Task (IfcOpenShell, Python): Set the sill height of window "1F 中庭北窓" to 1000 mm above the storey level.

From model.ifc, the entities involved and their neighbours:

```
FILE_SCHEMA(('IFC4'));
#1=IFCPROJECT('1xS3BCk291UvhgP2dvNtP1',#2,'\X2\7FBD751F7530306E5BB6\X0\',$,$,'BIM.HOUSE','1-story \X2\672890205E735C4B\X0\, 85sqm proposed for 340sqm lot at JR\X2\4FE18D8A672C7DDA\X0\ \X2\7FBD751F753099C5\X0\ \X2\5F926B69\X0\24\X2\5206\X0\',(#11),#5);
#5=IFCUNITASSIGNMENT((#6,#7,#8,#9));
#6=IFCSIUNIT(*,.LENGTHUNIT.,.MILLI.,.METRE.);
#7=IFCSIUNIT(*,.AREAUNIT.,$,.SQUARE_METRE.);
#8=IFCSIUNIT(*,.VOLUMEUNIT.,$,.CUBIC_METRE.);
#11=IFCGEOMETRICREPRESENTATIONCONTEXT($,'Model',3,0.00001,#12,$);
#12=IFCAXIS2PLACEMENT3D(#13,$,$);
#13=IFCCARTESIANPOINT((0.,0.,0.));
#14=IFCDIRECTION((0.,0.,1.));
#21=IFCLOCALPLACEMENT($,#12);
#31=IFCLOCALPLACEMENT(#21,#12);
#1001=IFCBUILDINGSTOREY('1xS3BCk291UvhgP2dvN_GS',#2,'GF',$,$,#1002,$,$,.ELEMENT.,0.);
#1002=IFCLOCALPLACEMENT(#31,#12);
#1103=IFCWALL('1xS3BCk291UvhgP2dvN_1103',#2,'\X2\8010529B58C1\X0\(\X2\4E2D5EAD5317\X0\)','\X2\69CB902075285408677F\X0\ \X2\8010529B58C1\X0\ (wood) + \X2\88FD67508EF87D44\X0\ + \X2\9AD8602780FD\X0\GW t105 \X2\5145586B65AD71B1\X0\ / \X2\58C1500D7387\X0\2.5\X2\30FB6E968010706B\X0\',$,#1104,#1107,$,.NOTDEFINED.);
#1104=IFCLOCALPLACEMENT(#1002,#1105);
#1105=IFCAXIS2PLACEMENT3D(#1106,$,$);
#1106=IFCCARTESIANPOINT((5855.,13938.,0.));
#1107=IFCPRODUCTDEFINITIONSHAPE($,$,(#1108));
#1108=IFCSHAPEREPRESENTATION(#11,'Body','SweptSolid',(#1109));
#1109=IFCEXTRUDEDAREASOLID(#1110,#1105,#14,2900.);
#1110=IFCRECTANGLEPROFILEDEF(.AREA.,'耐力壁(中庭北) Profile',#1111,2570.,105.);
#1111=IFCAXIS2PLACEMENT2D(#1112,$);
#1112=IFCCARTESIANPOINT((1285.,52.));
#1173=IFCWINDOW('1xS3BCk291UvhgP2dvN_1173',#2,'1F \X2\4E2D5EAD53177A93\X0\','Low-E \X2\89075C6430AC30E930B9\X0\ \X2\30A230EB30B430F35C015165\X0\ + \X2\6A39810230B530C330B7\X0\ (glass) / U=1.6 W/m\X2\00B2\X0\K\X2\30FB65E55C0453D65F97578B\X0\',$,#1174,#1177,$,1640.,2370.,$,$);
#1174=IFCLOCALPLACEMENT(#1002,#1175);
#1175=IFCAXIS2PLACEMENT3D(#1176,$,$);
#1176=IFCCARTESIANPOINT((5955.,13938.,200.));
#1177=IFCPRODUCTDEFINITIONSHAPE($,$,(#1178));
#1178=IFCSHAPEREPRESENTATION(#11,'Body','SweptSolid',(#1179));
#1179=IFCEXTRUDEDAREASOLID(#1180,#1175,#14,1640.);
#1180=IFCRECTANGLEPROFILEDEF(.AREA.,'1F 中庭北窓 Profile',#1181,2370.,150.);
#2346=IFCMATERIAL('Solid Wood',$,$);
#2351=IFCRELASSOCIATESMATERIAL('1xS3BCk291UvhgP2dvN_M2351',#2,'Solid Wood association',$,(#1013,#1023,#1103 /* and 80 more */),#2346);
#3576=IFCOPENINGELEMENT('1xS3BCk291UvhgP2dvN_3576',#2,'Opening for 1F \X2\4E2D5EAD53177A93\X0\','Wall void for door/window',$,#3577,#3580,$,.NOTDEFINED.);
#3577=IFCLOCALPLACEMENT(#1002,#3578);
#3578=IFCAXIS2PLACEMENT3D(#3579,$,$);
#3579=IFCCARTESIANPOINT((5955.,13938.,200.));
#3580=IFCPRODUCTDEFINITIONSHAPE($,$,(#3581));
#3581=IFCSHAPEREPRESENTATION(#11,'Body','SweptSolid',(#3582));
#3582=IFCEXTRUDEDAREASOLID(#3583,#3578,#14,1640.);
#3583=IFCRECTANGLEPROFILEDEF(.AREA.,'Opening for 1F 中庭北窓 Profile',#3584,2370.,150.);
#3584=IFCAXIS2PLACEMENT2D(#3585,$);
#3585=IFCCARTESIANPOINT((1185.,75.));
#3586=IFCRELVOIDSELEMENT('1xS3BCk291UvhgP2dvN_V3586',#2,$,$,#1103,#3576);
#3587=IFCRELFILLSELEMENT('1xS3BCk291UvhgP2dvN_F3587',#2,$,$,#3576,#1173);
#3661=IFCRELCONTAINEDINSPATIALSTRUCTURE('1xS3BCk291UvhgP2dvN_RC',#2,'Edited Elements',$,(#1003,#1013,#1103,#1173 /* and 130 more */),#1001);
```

```python
import numpy as np
import ifcopenshell
import ifcopenshell.api.geometry
import ifcopenshell.geom
import ifcopenshell.util.element
import ifcopenshell.util.placement
import ifcopenshell.util.shape
import ifcopenshell.util.unit

model = ifcopenshell.open("model.ifc")
unit_scale = ifcopenshell.util.unit.calculate_unit_scale(model)

window = model.by_guid("1xS3BCk291UvhgP2dvN_1173")
opening = window.FillsVoids[0].RelatingOpeningElement
storey = ifcopenshell.util.element.get_container(window, ifc_class="IfcBuildingStorey")
level = ifcopenshell.util.placement.get_local_placement(storey.ObjectPlacement)[2, 3]

# The opening's origin need not be at the sill, so measure its lowest point.
shape = ifcopenshell.geom.create_shape(ifcopenshell.geom.settings(), opening)
bottom = ifcopenshell.util.shape.get_shape_bottom_elevation(shape, shape.geometry) / unit_scale
dz = level + 1 / unit_scale - bottom

shift = np.array([0.0, 0.0, dz])
# The window is not placed relative to its opening, so move both.
for product in (opening, window):
    matrix = ifcopenshell.util.placement.get_local_placement(product.ObjectPlacement)
    matrix[:3, 3] += shift
    ifcopenshell.api.geometry.edit_object_placement(model, product=product, matrix=matrix, is_si=False)

print(f"moved by {dz * unit_scale:+.3f} m")

model.write("model_v2.ifc")
```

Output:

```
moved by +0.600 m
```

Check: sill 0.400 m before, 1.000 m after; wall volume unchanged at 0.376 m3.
